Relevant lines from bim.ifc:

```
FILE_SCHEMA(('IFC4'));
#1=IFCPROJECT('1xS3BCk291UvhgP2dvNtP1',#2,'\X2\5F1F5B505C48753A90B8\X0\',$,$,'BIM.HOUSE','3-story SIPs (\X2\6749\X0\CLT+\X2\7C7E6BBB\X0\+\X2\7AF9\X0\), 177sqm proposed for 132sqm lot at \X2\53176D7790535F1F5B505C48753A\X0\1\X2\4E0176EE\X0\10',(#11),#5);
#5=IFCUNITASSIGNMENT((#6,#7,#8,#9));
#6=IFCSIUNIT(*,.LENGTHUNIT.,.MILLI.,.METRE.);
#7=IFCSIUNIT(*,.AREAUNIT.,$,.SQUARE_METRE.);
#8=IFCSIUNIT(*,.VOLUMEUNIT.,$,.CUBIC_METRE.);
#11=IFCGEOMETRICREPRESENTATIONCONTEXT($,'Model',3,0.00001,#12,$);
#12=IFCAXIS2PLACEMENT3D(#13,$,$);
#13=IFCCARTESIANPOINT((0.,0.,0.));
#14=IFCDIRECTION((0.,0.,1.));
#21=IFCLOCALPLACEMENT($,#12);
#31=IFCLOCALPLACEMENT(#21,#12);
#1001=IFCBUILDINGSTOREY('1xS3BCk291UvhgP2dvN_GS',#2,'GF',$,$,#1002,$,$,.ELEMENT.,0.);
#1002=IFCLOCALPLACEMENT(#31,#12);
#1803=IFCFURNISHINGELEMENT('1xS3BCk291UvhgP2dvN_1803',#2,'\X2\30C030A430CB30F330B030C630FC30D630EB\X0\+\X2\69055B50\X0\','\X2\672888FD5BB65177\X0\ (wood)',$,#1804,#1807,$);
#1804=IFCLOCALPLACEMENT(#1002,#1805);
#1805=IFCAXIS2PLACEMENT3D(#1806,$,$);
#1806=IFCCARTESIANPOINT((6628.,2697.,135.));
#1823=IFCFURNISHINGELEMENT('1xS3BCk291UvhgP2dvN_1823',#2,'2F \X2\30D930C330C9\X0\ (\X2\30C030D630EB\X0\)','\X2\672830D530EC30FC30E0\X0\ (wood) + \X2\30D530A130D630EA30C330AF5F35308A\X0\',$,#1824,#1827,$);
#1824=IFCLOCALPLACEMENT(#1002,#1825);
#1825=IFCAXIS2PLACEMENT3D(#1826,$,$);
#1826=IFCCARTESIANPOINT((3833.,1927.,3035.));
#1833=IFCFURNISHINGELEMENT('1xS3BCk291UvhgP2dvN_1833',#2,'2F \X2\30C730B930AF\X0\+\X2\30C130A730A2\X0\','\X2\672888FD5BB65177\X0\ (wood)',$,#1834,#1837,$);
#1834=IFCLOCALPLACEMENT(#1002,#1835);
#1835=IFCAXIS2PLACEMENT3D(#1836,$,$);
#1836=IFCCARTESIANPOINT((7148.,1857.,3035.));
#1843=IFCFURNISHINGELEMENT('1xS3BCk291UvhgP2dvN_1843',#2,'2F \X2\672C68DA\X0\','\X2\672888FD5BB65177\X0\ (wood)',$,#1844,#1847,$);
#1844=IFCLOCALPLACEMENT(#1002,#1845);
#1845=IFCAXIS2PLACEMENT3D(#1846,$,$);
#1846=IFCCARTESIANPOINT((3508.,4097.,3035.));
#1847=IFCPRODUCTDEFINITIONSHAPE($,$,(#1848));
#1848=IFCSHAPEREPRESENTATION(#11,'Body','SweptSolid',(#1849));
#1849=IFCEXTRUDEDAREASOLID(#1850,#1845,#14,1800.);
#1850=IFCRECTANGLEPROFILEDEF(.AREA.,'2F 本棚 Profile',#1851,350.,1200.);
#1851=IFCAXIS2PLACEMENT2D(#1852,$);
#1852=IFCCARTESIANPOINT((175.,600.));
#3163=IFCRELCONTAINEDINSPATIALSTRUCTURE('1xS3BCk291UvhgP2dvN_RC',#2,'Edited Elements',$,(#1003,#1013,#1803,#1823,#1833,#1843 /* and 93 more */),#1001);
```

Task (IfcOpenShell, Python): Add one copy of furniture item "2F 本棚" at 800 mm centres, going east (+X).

```python
import numpy as np
import ifcopenshell
import ifcopenshell.api.geometry
import ifcopenshell.api.root
import ifcopenshell.util.element
import ifcopenshell.util.placement

model = ifcopenshell.open("bim.ifc")


def reuse_history(source, copy):
    """copy_class also copies each property set's owner history, people and application; keep the originals."""
    for rel in copy.IsDefinedBy:
        if rel.is_a("IfcRelDefinesByProperties") and (history := rel.RelatingPropertyDefinition.OwnerHistory):
            rel.RelatingPropertyDefinition.OwnerHistory = source.OwnerHistory
            ifcopenshell.util.element.remove_deep2(model, history)


source = model.by_guid("1xS3BCk291UvhgP2dvN_1843")
base = ifcopenshell.util.placement.get_local_placement(source.ObjectPlacement)
step = np.array([1.0, 0.0, 0.0]) * 800.0

for i in range(1, 2):
    copy = ifcopenshell.api.root.copy_class(model, product=source)
    copy.Representation = ifcopenshell.util.element.copy_deep(
        model, source.Representation, exclude=["IfcGeometricRepresentationContext", "IfcRepresentationMap"]
    )
    reuse_history(source, copy)
    matrix = base.copy()
    matrix[:3, 3] += i * step
    print("added at", matrix[:3, 3].round(3) + 0.0)
    ifcopenshell.api.geometry.edit_object_placement(model, product=copy, matrix=matrix, is_si=False)

model.write("bim_v2.ifc")
```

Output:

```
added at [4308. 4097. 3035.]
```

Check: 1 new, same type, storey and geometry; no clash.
